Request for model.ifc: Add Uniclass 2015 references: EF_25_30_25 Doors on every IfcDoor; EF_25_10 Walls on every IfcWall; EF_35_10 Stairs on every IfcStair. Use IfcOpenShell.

First a look at what the model holds.

```python
import ifcopenshell

model = ifcopenshell.open("model.ifc")
print(model.schema)
print("classifications:", [c.Name for c in model.by_type("IfcClassification")])
for ifc_class in ("IfcDoor", "IfcRoof", "IfcStair", "IfcWall", "IfcWindow"):
    print(ifc_class, len(model.by_type(ifc_class)))
```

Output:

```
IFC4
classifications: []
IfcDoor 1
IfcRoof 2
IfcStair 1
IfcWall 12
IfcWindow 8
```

```python
import ifcopenshell
import ifcopenshell.api.classification

model = ifcopenshell.open("model.ifc")

system = ifcopenshell.api.classification.add_classification(model, classification="Uniclass 2015")

codes = {
    "IfcDoor": ("EF_25_30_25", "Doors"),
    "IfcWall": ("EF_25_10", "Walls"),
    "IfcStair": ("EF_35_10", "Stairs"),
}
for ifc_class, (code, name) in codes.items():
    products = model.by_type(ifc_class)
    ifcopenshell.api.classification.add_reference(
        model, products=products, classification=system, identification=code, name=name
    )
    print(code, len(products))

model.write("model_updated.ifc")
```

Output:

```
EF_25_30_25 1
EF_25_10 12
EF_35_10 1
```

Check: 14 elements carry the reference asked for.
